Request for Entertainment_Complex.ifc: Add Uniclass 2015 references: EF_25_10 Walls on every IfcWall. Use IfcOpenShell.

First a look at what the model holds.

```python
import ifcopenshell

model = ifcopenshell.open("Entertainment_Complex.ifc")
print(model.schema)
print("classifications:", [c.Name for c in model.by_type("IfcClassification")])
for ifc_class in ("IfcDoor", "IfcRoof", "IfcStair", "IfcWall", "IfcWindow"):
    print(ifc_class, len(model.by_type(ifc_class)))
```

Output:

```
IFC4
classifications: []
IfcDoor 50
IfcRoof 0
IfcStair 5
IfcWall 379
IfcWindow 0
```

```python
import ifcopenshell
import ifcopenshell.api.classification

model = ifcopenshell.open("Entertainment_Complex.ifc")

system = ifcopenshell.api.classification.add_classification(model, classification="Uniclass 2015")

codes = {
    "IfcWall": ("EF_25_10", "Walls"),
}
for ifc_class, (code, name) in codes.items():
    products = model.by_type(ifc_class)
    ifcopenshell.api.classification.add_reference(
        model, products=products, classification=system, identification=code, name=name
    )
    print(code, len(products))

model.write("Entertainment_Complex_v2.ifc")
```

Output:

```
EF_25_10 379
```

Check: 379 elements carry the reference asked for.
